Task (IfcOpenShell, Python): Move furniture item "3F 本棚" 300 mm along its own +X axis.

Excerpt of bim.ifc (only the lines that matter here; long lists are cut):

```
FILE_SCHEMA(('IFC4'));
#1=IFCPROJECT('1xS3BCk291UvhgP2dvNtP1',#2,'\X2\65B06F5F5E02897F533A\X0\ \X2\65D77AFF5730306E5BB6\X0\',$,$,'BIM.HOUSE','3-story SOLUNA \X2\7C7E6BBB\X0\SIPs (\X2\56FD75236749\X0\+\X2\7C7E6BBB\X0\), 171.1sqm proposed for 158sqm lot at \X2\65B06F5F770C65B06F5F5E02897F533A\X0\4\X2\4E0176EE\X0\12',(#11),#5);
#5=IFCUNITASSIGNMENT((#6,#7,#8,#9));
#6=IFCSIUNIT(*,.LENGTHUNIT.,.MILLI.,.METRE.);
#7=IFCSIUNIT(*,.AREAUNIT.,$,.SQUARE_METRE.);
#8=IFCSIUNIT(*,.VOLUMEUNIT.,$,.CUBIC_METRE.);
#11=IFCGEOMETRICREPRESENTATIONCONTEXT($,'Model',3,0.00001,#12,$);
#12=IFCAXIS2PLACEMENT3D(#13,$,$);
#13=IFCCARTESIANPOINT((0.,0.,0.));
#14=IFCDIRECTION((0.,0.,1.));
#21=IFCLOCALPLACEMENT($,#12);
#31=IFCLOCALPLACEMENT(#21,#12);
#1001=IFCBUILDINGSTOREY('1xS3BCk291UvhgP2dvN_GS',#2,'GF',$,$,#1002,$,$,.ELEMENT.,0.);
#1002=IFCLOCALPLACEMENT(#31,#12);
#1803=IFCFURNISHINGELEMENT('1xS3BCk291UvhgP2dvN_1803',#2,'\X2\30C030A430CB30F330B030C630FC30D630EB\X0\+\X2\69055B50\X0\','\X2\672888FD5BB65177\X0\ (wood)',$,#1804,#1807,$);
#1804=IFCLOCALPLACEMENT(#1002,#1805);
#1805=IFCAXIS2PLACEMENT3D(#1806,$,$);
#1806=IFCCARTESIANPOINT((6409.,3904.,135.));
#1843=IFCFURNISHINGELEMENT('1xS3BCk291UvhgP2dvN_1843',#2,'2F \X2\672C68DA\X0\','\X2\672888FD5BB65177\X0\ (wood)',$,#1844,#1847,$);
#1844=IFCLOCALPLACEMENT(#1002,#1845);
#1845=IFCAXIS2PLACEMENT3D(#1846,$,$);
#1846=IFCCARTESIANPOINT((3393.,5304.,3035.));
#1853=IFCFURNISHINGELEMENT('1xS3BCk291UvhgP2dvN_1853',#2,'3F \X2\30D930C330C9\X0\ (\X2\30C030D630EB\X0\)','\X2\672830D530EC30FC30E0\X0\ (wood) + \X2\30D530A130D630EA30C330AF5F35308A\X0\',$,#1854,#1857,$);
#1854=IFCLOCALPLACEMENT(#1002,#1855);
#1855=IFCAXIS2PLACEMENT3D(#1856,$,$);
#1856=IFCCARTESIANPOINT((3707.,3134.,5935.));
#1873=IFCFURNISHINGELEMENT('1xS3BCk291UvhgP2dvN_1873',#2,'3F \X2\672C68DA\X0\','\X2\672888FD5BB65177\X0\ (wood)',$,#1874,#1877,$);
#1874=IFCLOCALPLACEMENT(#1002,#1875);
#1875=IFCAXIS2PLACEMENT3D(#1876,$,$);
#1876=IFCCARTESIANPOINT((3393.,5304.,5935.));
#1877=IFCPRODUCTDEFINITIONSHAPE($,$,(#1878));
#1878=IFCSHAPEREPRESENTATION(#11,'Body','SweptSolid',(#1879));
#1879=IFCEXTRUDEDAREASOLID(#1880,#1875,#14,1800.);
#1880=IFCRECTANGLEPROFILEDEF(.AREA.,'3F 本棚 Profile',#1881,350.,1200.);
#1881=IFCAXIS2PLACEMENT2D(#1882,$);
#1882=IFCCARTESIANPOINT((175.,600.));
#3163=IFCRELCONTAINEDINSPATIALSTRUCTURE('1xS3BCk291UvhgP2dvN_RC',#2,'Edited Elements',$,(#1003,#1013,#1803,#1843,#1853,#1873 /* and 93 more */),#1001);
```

```python
import ifcopenshell
import ifcopenshell.api.geometry
import ifcopenshell.util.placement
import ifcopenshell.util.unit

model = ifcopenshell.open("bim.ifc")
unit_scale = ifcopenshell.util.unit.calculate_unit_scale(model)

item = model.by_id(1873)
matrix = ifcopenshell.util.placement.get_local_placement(item.ObjectPlacement)
matrix[:3, 3] += matrix[:3, 0] * 0.3 / unit_scale
ifcopenshell.api.geometry.edit_object_placement(model, product=item, matrix=matrix, is_si=False)

print(ifcopenshell.util.placement.get_local_placement(item.ObjectPlacement).round(3) + 0.0)

model.write("bim_v2.ifc")
```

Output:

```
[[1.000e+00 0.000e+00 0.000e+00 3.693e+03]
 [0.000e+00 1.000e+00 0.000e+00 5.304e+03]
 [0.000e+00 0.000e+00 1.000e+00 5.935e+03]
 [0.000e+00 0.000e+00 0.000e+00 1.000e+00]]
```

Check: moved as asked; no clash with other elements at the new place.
